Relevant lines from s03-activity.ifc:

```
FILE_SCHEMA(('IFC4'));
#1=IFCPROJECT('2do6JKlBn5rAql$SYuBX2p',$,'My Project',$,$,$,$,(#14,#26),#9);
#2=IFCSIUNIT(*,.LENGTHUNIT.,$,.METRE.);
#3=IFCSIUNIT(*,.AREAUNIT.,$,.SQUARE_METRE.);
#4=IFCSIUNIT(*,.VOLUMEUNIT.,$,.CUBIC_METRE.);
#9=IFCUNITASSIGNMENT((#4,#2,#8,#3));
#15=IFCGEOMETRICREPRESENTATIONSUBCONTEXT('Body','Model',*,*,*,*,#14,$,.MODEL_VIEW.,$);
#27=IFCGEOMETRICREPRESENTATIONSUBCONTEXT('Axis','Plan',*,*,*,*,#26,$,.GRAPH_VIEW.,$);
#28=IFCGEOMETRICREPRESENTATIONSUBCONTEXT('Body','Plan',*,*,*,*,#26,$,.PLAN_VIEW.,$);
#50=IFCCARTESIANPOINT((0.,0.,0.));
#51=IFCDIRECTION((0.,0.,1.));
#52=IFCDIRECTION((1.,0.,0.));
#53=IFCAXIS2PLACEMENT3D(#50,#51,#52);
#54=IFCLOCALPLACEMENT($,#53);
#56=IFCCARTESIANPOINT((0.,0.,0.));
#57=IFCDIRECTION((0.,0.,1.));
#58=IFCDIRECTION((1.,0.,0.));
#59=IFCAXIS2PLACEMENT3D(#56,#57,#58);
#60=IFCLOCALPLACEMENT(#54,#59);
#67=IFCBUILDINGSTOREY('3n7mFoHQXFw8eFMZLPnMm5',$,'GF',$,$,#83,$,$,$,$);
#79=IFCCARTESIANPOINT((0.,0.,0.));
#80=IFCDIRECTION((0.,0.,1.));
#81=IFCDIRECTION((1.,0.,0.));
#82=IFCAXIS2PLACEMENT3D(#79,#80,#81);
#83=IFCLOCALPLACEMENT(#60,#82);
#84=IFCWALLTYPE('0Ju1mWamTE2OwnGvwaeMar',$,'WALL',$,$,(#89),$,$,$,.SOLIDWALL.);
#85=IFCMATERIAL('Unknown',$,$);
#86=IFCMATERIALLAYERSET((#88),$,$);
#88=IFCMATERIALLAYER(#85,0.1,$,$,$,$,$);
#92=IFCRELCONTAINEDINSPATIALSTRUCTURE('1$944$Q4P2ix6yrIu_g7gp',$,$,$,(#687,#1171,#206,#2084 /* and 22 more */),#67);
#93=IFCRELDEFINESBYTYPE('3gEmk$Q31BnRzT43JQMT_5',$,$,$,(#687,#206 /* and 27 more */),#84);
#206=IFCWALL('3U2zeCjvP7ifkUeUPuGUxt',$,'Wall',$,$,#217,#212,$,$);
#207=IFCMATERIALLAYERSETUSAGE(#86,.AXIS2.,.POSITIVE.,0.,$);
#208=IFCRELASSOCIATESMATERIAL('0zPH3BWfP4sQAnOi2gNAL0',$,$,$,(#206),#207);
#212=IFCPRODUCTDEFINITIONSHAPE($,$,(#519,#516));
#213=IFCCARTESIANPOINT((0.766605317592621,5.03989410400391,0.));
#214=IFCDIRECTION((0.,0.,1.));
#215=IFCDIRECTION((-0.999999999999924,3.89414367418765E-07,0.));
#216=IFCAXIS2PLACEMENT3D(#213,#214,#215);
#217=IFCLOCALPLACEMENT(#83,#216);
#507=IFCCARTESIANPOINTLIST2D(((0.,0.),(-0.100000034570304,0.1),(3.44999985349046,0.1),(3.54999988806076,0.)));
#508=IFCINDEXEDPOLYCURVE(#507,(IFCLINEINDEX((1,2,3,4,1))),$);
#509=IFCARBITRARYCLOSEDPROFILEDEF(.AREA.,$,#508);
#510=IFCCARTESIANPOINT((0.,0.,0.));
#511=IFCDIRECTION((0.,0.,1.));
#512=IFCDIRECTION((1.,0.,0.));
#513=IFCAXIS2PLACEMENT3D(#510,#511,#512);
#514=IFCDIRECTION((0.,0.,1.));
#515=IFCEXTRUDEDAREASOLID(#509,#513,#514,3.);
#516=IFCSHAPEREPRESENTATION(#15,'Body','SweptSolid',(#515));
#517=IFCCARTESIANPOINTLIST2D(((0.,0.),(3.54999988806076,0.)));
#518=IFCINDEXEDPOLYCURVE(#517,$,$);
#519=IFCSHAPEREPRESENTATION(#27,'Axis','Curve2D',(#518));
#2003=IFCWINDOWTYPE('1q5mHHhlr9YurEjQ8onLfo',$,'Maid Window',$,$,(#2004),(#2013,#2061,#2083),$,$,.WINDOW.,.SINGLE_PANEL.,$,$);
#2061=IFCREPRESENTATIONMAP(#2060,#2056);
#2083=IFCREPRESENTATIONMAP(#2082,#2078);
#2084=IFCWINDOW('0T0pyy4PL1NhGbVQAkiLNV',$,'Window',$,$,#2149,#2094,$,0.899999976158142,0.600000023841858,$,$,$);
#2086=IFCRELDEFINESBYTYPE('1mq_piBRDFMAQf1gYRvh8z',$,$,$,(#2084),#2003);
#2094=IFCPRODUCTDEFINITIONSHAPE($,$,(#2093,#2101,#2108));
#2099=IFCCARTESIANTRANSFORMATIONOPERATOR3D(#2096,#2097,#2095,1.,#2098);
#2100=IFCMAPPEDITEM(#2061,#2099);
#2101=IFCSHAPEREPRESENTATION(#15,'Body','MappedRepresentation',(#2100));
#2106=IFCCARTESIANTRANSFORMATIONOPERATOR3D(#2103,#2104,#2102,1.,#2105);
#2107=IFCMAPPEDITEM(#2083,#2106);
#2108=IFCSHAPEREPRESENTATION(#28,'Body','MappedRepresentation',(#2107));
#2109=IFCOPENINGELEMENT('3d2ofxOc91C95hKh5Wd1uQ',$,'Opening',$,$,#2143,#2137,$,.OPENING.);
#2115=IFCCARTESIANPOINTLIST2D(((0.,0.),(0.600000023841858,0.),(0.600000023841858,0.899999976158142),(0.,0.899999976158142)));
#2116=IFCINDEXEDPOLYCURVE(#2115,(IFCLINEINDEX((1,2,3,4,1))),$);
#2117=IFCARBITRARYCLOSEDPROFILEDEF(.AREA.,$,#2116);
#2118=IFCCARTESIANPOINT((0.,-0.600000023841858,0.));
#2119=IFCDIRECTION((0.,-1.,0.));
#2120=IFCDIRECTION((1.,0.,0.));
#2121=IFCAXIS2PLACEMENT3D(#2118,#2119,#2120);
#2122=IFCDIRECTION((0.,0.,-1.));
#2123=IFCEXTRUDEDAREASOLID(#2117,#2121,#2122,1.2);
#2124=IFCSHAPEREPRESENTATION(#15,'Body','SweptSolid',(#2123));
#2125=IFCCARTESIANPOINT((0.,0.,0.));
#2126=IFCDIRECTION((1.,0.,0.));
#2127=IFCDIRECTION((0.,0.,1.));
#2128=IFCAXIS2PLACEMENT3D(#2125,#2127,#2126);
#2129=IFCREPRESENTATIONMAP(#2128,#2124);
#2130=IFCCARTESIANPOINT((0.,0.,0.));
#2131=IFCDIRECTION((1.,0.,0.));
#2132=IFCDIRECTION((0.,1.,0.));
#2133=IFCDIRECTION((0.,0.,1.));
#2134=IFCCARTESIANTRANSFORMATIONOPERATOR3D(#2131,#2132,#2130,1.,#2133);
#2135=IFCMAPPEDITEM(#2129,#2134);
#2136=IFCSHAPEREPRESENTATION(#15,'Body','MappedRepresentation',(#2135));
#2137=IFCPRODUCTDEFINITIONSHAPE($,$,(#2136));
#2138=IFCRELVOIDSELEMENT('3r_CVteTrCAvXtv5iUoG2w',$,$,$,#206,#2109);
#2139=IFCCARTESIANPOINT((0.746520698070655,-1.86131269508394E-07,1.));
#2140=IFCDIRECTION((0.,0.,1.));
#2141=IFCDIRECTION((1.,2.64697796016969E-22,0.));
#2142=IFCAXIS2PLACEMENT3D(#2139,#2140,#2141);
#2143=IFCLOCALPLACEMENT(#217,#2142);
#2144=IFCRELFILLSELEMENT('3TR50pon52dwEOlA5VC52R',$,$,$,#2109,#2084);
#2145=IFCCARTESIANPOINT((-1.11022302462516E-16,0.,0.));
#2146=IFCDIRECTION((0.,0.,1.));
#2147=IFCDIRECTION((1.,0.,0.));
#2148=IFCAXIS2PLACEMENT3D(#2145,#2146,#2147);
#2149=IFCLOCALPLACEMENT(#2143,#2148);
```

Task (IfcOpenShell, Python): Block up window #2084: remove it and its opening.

```python
import ifcopenshell
import ifcopenshell.api.feature
import ifcopenshell.api.root
import ifcopenshell.geom
import ifcopenshell.util.shape

model = ifcopenshell.open("s03-activity.ifc")
settings = ifcopenshell.geom.settings()


def volume(element):
    """Net volume in cubic metres, openings subtracted."""
    shape = ifcopenshell.geom.create_shape(settings, element)
    return ifcopenshell.util.shape.get_volume(shape.geometry)


window = model.by_guid("0T0pyy4PL1NhGbVQAkiLNV")
opening = window.FillsVoids[0].RelatingOpeningElement
wall = opening.VoidsElements[0].RelatingBuildingElement
before = volume(wall)

ifcopenshell.api.root.remove_product(model, product=window)
ifcopenshell.api.feature.remove_feature(model, feature=opening)

after = volume(wall)

print(f"wall volume {before:.3f} -> {after:.3f} m3")

model.write("s03-activity_updated.ifc")
```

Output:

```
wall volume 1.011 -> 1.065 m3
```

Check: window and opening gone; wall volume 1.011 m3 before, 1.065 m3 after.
